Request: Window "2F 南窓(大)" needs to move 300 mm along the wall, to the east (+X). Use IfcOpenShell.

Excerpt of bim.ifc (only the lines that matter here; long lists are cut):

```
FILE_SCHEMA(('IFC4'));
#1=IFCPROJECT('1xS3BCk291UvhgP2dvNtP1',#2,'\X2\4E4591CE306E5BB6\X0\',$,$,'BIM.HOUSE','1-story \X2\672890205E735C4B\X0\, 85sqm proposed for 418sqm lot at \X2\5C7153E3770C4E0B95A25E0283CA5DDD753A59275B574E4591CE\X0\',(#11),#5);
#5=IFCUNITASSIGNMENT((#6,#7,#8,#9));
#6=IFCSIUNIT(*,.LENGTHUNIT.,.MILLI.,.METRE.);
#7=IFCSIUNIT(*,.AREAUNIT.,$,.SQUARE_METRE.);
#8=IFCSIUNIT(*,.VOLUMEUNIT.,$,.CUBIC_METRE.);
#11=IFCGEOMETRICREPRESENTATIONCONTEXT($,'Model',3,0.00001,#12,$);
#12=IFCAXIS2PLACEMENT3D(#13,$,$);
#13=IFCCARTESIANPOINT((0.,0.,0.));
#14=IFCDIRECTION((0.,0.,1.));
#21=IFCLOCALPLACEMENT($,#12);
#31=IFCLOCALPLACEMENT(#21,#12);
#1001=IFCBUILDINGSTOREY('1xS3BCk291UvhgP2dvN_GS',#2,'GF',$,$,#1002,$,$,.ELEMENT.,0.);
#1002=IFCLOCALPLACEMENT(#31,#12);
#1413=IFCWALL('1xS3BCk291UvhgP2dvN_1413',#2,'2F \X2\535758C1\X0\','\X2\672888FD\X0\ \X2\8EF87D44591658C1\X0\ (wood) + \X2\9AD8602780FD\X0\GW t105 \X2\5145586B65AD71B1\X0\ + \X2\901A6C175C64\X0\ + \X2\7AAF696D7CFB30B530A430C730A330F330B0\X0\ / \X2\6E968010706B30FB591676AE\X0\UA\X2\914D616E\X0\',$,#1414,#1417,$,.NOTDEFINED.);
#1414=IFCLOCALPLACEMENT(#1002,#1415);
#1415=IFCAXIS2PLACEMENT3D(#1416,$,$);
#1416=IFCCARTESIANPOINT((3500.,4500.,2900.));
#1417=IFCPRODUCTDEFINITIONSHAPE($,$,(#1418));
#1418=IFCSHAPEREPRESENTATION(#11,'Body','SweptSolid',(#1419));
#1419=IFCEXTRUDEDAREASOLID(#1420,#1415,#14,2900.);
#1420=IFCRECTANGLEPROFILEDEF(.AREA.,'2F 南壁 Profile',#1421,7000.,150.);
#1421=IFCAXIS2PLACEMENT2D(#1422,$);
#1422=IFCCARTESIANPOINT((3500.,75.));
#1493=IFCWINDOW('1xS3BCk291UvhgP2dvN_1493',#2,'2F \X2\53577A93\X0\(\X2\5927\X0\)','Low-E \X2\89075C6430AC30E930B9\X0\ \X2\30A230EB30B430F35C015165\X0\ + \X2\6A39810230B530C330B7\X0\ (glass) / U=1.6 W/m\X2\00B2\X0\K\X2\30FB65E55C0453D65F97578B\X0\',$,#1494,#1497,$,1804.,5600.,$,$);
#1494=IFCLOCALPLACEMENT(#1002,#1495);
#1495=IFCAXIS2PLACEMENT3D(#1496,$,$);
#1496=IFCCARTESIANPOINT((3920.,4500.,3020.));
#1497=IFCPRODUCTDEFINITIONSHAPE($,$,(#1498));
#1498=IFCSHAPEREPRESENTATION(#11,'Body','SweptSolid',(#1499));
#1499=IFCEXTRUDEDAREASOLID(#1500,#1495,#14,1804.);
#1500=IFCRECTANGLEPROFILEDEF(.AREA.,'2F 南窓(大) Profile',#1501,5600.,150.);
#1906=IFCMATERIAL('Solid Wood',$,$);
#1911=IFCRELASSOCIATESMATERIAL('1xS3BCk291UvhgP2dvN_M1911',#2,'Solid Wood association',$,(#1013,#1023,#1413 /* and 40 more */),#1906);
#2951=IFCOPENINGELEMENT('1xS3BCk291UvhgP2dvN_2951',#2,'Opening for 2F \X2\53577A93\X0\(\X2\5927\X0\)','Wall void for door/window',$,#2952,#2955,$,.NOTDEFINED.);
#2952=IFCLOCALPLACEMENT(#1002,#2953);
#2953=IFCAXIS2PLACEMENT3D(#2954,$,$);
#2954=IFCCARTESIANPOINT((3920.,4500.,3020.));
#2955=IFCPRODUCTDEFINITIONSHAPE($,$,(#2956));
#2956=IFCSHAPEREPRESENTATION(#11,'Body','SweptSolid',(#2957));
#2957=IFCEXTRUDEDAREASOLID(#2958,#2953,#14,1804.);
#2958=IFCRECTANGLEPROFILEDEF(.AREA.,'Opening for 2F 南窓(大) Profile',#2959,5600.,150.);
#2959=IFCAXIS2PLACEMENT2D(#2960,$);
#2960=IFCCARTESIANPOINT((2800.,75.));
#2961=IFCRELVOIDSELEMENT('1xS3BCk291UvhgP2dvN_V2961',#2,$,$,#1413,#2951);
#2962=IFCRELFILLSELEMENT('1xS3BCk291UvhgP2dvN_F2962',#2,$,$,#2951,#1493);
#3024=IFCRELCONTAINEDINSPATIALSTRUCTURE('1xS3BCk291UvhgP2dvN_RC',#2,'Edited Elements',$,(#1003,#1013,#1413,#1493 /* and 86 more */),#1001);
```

```python
import ifcopenshell
import ifcopenshell.api.geometry
import ifcopenshell.util.placement
import ifcopenshell.util.unit

model = ifcopenshell.open("bim.ifc")
unit_scale = ifcopenshell.util.unit.calculate_unit_scale(model)

window = model.by_guid("1xS3BCk291UvhgP2dvN_1493")
opening = window.FillsVoids[0].RelatingOpeningElement
wall = opening.VoidsElements[0].RelatingBuildingElement

wall_matrix = ifcopenshell.util.placement.get_local_placement(wall.ObjectPlacement)
shift = wall_matrix[:3, 0] * 0.3 / unit_scale
before = ifcopenshell.util.placement.get_local_placement(window.ObjectPlacement)[:3, 3].copy()

# The window is not placed relative to its opening, so move both.
for product in (opening, window):
    matrix = ifcopenshell.util.placement.get_local_placement(product.ObjectPlacement)
    matrix[:3, 3] += shift
    ifcopenshell.api.geometry.edit_object_placement(model, product=product, matrix=matrix, is_si=False)

after = ifcopenshell.util.placement.get_local_placement(window.ObjectPlacement)[:3, 3]
print("window moved by", (after - before).round(3) + 0.0)

model.write("bim_edited.ifc")
```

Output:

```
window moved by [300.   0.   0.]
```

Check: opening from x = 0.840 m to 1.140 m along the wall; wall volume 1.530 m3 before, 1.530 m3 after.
